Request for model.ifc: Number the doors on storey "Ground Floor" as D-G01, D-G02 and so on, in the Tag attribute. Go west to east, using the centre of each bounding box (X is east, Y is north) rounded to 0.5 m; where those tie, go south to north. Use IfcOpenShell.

First a look at what the model holds.

```python
import ifcopenshell
import ifcopenshell.util.element
import ifcopenshell.util.placement

model = ifcopenshell.open("model.ifc")
print(model.schema)
storey = next(s for s in model.by_type("IfcBuildingStorey") if s.Name == "Ground Floor")
doors = [e for e in ifcopenshell.util.element.get_decomposition(storey) if e.is_a("IfcDoor")]
for e in sorted(doors, key=lambda e: e.id()):
    origin = ifcopenshell.util.placement.get_local_placement(e.ObjectPlacement)[:3, 3]
    print(e.id(), e.Tag, e.Name, origin.round(2) + 0.0, sep=" | ")
```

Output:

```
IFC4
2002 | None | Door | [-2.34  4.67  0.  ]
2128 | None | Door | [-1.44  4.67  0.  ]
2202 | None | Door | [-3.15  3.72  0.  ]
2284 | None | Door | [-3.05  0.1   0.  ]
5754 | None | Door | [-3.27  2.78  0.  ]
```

```python
import ifcopenshell
import ifcopenshell.geom
import ifcopenshell.util.element
import ifcopenshell.util.shape

model = ifcopenshell.open("model.ifc")
settings = ifcopenshell.geom.settings()
settings.set("use-world-coords", True)


def centre(element):
    shape = ifcopenshell.geom.create_shape(settings, element)
    return ifcopenshell.util.shape.get_bbox_centroid(shape.geometry)


storey = next(s for s in model.by_type("IfcBuildingStorey") if s.Name == "Ground Floor")
doors = [e for e in ifcopenshell.util.element.get_decomposition(storey) if e.is_a("IfcDoor")]

# Insertion points can sit at a corner or the storey origin, so sort by the geometry (in metres).
centres = {e: centre(e) for e in doors}
doors.sort(key=lambda e: (round(centres[e][0] / 0.5), centres[e][1]))

for i, e in enumerate(doors, start=1):
    number = f"D-G{i:02d}"
    e.Tag = number
    print(e.id(), number)

model.write("model_updated.ifc")
```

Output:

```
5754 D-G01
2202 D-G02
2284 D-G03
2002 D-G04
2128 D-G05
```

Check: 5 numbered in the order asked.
